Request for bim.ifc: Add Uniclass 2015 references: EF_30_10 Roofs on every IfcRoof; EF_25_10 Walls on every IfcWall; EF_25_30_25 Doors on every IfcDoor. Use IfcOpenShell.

First a look at what the model holds.

```python
import ifcopenshell

model = ifcopenshell.open("bim.ifc")
print(model.schema)
print("classifications:", [c.Name for c in model.by_type("IfcClassification")])
for ifc_class in ("IfcDoor", "IfcRoof", "IfcStair", "IfcWall", "IfcWindow"):
    print(ifc_class, len(model.by_type(ifc_class)))
```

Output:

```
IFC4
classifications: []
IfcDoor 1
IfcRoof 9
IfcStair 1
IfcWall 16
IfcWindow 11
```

```python
import ifcopenshell
import ifcopenshell.api.classification

model = ifcopenshell.open("bim.ifc")

system = ifcopenshell.api.classification.add_classification(model, classification="Uniclass 2015")

codes = {
    "IfcRoof": ("EF_30_10", "Roofs"),
    "IfcWall": ("EF_25_10", "Walls"),
    "IfcDoor": ("EF_25_30_25", "Doors"),
}
for ifc_class, (code, name) in codes.items():
    products = model.by_type(ifc_class)
    ifcopenshell.api.classification.add_reference(
        model, products=products, classification=system, identification=code, name=name
    )
    print(code, len(products))

model.write("bim_edited.ifc")
```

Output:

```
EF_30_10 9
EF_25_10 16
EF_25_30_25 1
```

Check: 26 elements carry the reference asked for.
